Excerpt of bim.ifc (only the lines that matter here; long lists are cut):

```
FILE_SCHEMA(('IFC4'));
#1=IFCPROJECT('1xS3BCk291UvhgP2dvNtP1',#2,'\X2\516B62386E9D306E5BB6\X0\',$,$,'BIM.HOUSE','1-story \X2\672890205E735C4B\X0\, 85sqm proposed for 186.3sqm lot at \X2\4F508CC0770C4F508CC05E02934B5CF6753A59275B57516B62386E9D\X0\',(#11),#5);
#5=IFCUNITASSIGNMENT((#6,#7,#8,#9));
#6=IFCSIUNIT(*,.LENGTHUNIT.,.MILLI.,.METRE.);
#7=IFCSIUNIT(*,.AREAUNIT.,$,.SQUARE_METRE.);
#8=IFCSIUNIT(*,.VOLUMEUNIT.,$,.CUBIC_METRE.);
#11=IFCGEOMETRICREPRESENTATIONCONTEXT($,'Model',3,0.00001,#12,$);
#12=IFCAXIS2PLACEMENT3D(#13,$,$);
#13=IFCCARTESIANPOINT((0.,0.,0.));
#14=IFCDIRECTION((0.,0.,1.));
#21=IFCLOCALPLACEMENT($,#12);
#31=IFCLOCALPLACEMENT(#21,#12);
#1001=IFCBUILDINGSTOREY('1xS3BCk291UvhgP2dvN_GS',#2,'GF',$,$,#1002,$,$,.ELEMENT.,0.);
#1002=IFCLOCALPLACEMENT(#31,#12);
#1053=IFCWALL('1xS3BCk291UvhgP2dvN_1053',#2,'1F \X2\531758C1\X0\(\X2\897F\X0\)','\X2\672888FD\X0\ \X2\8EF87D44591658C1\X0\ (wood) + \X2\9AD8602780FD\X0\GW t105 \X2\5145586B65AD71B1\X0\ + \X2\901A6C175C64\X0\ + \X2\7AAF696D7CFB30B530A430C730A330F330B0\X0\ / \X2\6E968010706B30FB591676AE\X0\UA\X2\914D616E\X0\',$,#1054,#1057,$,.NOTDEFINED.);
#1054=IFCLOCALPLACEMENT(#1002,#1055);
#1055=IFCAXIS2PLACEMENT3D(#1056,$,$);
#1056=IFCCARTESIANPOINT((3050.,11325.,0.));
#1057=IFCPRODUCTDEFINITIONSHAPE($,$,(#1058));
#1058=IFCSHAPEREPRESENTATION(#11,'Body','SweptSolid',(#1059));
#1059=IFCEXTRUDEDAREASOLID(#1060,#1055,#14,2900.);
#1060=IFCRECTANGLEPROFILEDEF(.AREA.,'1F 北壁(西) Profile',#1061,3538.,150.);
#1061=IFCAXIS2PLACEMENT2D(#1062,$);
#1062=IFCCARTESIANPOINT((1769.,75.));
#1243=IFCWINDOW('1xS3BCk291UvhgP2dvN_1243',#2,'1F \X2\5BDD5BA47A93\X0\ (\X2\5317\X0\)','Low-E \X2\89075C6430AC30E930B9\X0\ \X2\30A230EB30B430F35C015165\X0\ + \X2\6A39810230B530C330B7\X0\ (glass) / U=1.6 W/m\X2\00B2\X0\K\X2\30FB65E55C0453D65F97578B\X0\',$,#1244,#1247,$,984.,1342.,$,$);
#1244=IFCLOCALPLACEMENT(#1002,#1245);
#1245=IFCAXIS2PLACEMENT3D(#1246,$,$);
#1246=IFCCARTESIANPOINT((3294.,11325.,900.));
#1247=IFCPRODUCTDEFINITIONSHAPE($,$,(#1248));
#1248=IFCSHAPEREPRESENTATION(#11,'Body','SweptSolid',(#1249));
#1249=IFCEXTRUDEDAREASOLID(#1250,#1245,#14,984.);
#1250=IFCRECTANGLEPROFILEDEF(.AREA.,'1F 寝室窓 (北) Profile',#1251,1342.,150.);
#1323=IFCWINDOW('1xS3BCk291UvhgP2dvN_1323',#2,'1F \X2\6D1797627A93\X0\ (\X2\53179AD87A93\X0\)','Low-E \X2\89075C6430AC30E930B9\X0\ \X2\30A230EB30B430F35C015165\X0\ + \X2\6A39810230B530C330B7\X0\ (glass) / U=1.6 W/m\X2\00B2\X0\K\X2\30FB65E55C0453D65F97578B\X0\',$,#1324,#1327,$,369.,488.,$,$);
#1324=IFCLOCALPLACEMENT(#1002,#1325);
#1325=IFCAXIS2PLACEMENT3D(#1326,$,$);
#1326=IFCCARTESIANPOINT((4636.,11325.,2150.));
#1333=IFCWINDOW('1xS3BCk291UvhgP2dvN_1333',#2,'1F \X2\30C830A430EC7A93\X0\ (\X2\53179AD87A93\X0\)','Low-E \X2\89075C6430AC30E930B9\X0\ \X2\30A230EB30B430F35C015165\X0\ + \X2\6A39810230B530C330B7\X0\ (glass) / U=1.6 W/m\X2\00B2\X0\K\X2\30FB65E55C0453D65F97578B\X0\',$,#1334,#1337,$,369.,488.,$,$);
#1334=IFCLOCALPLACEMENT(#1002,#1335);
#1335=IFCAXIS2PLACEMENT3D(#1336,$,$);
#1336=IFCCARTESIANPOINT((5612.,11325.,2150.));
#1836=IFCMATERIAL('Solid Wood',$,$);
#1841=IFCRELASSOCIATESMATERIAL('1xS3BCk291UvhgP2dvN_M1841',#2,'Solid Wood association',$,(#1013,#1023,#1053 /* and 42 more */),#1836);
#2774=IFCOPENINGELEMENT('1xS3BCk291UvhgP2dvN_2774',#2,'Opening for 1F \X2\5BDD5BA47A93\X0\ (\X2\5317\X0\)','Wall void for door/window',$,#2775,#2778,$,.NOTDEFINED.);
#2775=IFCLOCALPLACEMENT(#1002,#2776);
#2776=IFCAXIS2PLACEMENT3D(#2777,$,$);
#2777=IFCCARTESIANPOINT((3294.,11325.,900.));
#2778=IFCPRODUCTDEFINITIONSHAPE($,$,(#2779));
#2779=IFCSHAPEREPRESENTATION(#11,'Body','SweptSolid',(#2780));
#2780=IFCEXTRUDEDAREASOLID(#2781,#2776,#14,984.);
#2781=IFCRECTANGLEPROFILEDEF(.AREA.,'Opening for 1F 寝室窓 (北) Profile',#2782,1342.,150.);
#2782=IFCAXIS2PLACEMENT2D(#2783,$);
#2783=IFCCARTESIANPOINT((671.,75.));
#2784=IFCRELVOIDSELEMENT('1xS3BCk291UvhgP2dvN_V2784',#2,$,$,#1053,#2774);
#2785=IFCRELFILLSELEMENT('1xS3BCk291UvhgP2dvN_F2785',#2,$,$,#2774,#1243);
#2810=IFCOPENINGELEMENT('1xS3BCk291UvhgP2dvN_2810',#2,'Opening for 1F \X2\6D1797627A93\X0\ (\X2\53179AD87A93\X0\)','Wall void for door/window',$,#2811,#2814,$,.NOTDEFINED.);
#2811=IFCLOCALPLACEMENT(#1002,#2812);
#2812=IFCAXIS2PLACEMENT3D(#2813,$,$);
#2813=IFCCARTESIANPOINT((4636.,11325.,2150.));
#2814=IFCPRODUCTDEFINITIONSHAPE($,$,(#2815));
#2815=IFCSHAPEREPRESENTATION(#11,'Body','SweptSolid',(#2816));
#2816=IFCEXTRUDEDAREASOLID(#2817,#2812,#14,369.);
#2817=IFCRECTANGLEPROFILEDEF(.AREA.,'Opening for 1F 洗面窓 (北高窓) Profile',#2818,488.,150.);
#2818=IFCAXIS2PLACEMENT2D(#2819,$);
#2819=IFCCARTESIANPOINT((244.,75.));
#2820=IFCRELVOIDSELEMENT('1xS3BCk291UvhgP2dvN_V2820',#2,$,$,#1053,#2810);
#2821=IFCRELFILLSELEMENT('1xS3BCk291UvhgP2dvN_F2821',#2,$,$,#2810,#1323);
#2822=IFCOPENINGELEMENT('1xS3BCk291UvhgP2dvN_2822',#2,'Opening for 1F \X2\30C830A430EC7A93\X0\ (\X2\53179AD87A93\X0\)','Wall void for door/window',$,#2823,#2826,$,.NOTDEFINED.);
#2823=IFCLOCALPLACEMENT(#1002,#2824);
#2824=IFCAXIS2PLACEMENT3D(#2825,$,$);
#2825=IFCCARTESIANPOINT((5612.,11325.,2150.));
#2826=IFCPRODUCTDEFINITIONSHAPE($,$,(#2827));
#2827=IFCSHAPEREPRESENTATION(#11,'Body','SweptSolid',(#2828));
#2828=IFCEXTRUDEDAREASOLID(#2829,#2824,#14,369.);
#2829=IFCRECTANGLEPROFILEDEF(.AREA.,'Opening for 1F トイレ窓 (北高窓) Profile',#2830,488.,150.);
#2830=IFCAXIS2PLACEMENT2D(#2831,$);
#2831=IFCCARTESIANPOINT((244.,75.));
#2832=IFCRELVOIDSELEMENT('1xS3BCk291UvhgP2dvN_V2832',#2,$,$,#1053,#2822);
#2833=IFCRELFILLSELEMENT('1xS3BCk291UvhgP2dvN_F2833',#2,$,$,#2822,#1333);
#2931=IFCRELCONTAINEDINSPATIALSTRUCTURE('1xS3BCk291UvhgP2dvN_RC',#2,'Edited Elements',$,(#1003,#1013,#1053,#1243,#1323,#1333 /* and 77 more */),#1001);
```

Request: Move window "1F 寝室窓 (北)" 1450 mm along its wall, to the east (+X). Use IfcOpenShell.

```python
import ifcopenshell
import ifcopenshell.api.geometry
import ifcopenshell.util.placement

model = ifcopenshell.open("bim.ifc")

window = model.by_id(1243)
opening = window.FillsVoids[0].RelatingOpeningElement
wall = opening.VoidsElements[0].RelatingBuildingElement

wall_matrix = ifcopenshell.util.placement.get_local_placement(wall.ObjectPlacement)
shift = wall_matrix[:3, 0] * 1450.0
before = ifcopenshell.util.placement.get_local_placement(window.ObjectPlacement)[:3, 3].copy()

# The window is not placed relative to its opening, so move both.
for product in (opening, window):
    matrix = ifcopenshell.util.placement.get_local_placement(product.ObjectPlacement)
    matrix[:3, 3] += shift
    ifcopenshell.api.geometry.edit_object_placement(model, product=product, matrix=matrix, is_si=False)

after = ifcopenshell.util.placement.get_local_placement(window.ObjectPlacement)[:3, 3]
print("window moved by", (after - before).round(3) + 0.0)

model.write("bim_edited.ifc")
```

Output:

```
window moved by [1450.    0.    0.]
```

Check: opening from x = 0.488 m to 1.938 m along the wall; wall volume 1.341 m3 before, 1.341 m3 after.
